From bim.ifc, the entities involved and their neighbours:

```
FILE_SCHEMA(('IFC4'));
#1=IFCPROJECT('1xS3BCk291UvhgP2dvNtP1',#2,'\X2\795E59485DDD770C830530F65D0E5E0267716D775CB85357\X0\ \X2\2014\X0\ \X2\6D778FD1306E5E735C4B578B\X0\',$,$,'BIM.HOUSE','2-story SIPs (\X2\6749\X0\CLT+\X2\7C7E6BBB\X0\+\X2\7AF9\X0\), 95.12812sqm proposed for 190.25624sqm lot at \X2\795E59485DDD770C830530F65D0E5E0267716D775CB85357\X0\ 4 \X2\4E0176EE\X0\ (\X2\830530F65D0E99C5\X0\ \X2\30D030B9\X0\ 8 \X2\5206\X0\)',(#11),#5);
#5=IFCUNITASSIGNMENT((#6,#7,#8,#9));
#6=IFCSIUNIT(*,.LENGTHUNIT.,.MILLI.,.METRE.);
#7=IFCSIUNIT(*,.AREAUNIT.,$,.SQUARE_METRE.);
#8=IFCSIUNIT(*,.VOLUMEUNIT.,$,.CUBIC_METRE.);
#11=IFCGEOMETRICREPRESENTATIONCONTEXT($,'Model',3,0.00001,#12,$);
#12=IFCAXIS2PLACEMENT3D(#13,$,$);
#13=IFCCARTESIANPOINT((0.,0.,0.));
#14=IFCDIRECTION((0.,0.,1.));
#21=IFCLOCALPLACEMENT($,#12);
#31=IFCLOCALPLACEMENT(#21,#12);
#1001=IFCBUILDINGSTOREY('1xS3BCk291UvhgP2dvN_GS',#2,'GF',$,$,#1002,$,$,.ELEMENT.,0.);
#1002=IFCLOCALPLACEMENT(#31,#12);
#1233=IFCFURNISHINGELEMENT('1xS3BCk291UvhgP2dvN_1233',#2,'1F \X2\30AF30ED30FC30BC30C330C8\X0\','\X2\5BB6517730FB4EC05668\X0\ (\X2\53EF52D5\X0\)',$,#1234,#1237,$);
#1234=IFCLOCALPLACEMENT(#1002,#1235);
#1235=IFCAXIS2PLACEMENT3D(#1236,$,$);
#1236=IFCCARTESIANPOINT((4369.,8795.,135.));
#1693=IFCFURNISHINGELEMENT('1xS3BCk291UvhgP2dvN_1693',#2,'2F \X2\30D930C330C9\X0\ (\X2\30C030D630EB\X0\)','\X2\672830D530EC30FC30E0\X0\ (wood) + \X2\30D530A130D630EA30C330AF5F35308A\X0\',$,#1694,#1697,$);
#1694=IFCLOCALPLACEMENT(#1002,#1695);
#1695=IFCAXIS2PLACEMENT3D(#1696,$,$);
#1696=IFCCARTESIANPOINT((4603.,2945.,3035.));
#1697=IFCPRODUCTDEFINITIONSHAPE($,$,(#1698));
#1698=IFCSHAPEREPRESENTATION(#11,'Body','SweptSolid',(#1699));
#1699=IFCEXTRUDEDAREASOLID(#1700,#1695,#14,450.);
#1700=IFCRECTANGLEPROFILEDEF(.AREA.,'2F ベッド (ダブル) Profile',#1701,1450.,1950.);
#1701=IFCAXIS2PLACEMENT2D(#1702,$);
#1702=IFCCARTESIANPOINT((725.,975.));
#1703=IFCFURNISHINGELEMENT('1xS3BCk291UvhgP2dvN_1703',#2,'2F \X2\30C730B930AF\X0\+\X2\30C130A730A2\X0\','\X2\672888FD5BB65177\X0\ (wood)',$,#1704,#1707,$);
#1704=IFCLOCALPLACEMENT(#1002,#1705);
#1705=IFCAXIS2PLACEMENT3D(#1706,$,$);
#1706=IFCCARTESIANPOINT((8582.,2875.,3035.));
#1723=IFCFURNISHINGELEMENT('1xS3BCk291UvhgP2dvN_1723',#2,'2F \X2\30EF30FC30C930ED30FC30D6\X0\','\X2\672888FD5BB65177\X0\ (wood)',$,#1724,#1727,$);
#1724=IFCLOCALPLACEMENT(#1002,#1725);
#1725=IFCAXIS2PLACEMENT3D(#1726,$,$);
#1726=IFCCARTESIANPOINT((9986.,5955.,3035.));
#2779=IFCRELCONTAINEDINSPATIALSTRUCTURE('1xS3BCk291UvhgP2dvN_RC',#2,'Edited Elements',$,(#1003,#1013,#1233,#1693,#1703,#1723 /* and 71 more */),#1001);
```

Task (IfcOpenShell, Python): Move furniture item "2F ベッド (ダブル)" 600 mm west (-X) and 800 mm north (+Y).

```python
import ifcopenshell
import ifcopenshell.api.geometry
import ifcopenshell.util.placement
import ifcopenshell.util.unit

model = ifcopenshell.open("bim.ifc")
unit_scale = ifcopenshell.util.unit.calculate_unit_scale(model)

item = model.by_guid("1xS3BCk291UvhgP2dvN_1693")
matrix = ifcopenshell.util.placement.get_local_placement(item.ObjectPlacement)
matrix[0, 3] -= 0.6 / unit_scale
matrix[1, 3] += 0.8 / unit_scale
ifcopenshell.api.geometry.edit_object_placement(model, product=item, matrix=matrix, is_si=False)

print(ifcopenshell.util.placement.get_local_placement(item.ObjectPlacement).round(3) + 0.0)

model.write("bim_edited.ifc")
```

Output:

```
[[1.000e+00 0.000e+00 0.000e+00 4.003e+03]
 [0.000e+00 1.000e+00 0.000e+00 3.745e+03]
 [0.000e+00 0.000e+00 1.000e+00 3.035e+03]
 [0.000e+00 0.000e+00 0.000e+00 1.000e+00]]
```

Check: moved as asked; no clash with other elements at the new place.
